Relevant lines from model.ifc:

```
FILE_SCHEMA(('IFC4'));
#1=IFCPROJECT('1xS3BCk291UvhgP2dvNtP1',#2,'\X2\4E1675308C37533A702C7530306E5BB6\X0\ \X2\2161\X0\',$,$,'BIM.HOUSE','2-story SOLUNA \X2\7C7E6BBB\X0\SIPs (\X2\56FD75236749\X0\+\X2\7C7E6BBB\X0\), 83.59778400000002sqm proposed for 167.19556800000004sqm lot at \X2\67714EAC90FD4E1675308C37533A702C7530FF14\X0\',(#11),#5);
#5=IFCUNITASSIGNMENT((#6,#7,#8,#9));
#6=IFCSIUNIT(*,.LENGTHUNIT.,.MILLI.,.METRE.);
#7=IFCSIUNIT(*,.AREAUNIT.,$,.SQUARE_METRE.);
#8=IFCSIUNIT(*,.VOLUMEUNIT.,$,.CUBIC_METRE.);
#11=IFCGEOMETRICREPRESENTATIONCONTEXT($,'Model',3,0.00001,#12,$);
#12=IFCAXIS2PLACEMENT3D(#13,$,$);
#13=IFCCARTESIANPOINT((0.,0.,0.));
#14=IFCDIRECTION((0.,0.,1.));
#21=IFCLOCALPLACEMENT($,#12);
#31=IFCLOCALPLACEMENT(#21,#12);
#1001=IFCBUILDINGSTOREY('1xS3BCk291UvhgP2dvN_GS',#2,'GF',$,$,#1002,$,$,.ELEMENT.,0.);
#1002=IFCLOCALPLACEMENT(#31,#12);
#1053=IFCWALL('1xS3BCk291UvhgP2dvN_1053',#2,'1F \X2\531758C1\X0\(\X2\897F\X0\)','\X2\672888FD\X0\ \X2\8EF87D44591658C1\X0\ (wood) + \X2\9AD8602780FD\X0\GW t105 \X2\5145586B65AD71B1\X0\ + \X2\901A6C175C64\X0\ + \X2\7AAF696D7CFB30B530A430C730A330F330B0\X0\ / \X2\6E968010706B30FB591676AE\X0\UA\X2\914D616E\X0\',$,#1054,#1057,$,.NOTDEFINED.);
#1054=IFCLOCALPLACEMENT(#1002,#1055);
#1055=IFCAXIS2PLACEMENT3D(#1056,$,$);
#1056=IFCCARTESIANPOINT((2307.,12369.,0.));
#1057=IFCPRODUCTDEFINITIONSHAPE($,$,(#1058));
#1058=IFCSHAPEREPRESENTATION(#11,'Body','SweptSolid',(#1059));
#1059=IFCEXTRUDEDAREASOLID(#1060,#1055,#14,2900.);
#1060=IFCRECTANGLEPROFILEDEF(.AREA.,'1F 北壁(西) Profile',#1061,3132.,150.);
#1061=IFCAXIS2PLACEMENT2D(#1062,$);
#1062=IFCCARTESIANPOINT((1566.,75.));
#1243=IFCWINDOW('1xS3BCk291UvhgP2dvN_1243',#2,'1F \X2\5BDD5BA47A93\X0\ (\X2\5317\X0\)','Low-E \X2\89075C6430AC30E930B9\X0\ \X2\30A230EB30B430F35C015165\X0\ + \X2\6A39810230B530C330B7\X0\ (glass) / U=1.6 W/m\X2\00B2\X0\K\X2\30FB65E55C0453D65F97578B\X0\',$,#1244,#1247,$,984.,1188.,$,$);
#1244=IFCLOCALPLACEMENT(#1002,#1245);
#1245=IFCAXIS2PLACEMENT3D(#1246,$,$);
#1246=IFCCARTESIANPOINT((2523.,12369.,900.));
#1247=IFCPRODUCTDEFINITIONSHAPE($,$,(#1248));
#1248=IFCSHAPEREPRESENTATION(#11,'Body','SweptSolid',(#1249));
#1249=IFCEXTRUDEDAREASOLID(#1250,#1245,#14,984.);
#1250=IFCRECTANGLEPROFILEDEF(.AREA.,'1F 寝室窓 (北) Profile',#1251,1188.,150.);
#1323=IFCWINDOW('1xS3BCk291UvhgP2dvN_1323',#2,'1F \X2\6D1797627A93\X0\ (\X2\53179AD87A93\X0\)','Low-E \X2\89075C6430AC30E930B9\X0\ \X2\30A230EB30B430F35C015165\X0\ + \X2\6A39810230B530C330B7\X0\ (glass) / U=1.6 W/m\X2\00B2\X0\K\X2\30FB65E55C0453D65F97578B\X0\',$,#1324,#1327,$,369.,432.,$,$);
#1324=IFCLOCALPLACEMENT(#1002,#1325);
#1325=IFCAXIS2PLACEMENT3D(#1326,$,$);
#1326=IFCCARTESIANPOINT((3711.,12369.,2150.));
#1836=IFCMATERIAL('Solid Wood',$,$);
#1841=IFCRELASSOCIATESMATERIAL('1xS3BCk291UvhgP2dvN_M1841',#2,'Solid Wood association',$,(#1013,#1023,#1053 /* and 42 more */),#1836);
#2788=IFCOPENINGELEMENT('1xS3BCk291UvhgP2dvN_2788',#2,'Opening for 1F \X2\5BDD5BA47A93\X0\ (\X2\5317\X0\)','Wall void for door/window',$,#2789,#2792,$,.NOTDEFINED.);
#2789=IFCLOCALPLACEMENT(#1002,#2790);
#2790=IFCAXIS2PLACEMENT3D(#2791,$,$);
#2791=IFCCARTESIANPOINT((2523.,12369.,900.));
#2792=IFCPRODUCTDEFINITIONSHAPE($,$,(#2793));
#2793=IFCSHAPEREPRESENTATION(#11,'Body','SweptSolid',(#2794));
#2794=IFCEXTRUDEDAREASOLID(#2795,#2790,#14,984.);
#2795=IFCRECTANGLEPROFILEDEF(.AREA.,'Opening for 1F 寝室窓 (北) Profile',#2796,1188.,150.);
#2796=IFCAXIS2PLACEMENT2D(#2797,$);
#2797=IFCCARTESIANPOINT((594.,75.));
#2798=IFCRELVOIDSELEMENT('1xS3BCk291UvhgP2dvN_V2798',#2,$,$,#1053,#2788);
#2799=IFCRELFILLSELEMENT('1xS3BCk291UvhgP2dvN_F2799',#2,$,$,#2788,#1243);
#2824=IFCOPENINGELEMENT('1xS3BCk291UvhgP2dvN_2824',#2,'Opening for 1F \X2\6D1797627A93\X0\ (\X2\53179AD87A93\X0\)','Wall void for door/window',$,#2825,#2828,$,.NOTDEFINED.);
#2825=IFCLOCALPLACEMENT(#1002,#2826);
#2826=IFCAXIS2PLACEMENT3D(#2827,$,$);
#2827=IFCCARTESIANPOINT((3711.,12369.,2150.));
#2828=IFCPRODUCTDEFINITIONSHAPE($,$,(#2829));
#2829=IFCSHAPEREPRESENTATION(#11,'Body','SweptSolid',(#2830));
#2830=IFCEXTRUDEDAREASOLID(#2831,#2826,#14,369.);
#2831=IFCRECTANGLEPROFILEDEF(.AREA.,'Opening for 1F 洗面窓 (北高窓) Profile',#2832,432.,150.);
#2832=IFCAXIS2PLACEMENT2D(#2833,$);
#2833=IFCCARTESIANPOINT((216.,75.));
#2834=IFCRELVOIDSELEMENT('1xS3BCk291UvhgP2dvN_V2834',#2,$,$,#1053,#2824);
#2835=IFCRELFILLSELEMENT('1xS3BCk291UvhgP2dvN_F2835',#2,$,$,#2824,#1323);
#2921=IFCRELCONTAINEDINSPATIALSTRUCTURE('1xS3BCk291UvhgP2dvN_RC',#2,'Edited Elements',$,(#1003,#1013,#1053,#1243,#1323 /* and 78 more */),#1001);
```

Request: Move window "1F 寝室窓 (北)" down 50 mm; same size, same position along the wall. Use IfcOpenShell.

```python
import numpy as np
import ifcopenshell
import ifcopenshell.api.geometry
import ifcopenshell.util.placement
import ifcopenshell.util.unit

model = ifcopenshell.open("model.ifc")
unit_scale = ifcopenshell.util.unit.calculate_unit_scale(model)

window = model.by_id(1243)
opening = window.FillsVoids[0].RelatingOpeningElement
dz = -0.05 / unit_scale

shift = np.array([0.0, 0.0, dz])
# The window is not placed relative to its opening, so move both.
for product in (opening, window):
    matrix = ifcopenshell.util.placement.get_local_placement(product.ObjectPlacement)
    matrix[:3, 3] += shift
    ifcopenshell.api.geometry.edit_object_placement(model, product=product, matrix=matrix, is_si=False)

print(f"moved by {dz * unit_scale:+.3f} m")

model.write("model_edited.ifc")
```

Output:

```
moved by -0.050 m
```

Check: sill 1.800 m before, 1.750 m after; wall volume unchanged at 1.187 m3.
